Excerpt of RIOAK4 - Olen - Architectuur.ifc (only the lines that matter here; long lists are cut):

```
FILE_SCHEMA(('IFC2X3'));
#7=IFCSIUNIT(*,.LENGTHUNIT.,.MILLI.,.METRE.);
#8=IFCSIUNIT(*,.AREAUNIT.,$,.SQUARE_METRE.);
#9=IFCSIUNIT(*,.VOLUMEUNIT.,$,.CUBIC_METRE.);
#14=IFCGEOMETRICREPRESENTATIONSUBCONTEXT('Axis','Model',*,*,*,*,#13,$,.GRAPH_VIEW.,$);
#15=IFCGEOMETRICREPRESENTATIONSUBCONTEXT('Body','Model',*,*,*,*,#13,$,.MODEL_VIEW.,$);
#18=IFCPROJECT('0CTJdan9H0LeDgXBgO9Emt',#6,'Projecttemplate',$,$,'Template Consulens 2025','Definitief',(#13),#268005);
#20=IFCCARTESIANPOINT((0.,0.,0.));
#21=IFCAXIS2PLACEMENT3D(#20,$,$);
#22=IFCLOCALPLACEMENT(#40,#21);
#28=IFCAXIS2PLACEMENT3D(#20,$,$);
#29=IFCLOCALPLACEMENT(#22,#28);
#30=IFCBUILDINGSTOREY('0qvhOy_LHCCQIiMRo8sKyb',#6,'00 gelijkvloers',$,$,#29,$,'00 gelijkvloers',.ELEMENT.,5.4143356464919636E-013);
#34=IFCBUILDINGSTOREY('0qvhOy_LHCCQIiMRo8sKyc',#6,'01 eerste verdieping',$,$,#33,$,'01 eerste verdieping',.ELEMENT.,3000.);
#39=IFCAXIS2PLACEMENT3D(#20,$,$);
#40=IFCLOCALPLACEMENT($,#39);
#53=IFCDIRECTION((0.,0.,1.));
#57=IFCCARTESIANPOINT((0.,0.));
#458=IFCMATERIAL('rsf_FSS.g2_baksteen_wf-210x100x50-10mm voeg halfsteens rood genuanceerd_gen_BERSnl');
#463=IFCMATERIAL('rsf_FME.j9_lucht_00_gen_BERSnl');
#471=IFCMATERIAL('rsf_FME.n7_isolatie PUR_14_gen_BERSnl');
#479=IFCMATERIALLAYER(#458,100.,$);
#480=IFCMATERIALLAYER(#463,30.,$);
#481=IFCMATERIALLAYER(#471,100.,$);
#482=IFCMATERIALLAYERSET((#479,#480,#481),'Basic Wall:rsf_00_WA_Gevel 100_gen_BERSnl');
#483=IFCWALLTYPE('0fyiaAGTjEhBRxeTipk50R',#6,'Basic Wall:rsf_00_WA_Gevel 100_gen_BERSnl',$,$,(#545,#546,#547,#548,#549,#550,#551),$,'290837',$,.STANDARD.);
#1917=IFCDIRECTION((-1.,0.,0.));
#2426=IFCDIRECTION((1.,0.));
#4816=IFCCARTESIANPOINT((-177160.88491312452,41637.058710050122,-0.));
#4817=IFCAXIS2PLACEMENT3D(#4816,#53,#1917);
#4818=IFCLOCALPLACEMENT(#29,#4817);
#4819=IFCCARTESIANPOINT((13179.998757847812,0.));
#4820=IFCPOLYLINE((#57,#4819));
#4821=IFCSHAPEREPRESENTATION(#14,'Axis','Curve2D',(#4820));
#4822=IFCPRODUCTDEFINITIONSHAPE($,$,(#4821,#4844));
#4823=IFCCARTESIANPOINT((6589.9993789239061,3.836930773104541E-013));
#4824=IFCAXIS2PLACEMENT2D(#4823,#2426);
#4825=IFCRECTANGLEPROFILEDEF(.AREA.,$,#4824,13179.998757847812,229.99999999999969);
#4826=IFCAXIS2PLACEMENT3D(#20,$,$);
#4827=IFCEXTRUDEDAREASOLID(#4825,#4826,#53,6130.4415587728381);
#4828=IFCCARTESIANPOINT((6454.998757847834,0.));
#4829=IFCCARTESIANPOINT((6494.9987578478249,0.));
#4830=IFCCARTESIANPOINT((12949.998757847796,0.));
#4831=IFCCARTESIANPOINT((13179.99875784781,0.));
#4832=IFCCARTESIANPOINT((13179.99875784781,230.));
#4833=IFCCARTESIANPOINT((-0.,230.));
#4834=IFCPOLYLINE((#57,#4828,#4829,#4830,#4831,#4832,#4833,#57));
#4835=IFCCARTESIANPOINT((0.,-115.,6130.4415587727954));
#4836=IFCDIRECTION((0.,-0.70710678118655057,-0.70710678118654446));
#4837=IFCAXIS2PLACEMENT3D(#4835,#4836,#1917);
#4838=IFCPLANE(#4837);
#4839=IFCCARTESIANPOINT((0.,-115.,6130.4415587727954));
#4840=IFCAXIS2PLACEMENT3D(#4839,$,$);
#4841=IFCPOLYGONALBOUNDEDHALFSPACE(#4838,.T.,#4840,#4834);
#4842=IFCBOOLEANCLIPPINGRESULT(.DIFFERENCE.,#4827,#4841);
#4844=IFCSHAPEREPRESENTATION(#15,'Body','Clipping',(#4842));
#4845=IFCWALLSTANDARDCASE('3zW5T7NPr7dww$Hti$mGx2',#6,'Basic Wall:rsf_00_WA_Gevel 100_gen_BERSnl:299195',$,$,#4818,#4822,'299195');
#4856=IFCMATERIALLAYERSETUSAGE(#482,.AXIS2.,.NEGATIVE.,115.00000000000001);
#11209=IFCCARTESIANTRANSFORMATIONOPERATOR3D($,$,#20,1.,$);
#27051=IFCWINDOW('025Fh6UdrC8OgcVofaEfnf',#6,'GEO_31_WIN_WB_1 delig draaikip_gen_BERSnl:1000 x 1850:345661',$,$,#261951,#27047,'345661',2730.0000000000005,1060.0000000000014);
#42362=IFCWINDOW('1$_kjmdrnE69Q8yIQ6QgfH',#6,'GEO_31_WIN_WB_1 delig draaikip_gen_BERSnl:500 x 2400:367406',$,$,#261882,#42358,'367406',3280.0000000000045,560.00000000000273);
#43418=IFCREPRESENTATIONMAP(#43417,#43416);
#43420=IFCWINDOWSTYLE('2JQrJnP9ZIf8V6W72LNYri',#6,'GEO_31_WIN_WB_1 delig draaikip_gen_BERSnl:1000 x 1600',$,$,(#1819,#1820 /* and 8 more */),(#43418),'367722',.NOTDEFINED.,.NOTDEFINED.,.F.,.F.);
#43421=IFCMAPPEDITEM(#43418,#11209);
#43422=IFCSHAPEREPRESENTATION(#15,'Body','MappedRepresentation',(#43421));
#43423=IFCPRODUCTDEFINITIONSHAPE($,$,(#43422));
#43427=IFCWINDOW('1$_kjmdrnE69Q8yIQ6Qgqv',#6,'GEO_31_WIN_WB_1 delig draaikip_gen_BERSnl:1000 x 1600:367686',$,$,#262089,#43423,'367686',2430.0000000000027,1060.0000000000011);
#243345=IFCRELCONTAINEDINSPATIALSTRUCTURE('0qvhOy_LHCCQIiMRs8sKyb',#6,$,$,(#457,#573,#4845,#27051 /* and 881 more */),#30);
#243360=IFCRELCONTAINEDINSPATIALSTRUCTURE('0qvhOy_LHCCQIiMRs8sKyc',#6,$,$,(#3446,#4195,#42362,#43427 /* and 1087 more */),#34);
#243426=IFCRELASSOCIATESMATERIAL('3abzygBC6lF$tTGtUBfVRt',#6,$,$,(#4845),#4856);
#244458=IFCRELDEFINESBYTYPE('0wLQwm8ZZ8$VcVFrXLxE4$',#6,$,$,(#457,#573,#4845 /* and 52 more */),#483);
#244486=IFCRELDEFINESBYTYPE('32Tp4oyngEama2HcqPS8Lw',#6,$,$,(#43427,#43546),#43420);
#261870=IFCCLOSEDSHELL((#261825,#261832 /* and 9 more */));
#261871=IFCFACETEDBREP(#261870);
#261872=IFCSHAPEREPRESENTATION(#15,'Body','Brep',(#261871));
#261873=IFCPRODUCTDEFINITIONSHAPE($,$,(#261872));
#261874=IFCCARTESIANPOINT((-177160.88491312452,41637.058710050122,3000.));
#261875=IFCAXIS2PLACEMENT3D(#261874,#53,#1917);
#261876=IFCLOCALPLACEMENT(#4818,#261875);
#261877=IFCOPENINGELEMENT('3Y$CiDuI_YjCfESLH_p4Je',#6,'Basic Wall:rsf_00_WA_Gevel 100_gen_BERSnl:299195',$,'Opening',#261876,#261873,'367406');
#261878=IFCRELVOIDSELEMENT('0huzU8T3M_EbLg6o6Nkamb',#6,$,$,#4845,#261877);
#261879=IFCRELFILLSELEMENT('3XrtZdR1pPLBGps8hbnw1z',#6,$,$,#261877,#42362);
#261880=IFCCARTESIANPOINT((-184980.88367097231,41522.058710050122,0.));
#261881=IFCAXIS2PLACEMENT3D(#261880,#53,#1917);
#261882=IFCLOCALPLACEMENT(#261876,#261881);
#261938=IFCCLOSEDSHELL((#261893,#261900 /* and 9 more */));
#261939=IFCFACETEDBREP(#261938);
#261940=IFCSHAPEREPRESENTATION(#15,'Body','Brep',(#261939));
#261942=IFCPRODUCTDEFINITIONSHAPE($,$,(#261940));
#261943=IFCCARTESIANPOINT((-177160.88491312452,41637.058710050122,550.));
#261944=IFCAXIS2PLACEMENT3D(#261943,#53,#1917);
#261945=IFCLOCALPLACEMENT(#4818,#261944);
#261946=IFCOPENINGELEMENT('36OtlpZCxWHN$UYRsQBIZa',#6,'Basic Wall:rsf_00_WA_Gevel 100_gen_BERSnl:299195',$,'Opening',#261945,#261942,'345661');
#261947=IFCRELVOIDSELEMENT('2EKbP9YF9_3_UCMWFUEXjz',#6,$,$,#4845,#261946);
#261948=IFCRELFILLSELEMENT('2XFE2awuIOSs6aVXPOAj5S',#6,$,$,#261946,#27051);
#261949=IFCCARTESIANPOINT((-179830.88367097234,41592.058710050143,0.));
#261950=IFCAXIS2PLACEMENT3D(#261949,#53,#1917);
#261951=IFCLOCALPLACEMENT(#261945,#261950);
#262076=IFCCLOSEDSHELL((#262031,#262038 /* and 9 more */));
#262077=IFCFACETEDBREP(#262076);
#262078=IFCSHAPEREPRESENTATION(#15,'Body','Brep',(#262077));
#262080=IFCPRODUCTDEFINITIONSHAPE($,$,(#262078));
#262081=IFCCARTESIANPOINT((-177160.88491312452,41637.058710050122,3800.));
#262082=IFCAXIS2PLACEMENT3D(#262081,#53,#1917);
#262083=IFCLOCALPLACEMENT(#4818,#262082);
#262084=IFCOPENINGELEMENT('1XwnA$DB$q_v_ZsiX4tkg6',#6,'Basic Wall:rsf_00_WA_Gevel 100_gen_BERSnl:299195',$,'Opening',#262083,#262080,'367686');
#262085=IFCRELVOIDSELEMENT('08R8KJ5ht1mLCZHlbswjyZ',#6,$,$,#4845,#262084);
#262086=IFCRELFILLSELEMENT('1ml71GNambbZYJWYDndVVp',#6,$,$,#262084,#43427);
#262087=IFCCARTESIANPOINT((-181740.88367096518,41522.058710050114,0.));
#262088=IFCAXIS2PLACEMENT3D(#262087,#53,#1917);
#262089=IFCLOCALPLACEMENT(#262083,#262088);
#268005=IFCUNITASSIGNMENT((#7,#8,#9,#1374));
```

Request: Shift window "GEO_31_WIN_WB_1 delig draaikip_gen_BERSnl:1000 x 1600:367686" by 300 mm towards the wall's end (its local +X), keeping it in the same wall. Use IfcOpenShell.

```python
import ifcopenshell
import ifcopenshell.api.geometry
import ifcopenshell.util.placement
import ifcopenshell.util.unit

model = ifcopenshell.open("RIOAK4 - Olen - Architectuur.ifc")
unit_scale = ifcopenshell.util.unit.calculate_unit_scale(model)

window = model.by_guid("1$_kjmdrnE69Q8yIQ6Qgqv")
opening = window.FillsVoids[0].RelatingOpeningElement
wall = opening.VoidsElements[0].RelatingBuildingElement

wall_matrix = ifcopenshell.util.placement.get_local_placement(wall.ObjectPlacement)
shift = wall_matrix[:3, 0] * 0.3 / unit_scale
before = ifcopenshell.util.placement.get_local_placement(window.ObjectPlacement)[:3, 3].copy()

# The window is placed relative to its opening, so it follows when the opening moves.
matrix = ifcopenshell.util.placement.get_local_placement(opening.ObjectPlacement)
matrix[:3, 3] += shift
ifcopenshell.api.geometry.edit_object_placement(
    model, product=opening, matrix=matrix, is_si=False, should_transform_children=True
)

after = ifcopenshell.util.placement.get_local_placement(window.ObjectPlacement)[:3, 3]
print("window moved by", (after - before).round(3) + 0.0)

model.write("RIOAK4 - Olen - Architectuur-out.ifc")
```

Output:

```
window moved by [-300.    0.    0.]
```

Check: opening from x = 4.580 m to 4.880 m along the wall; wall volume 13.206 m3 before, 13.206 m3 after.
